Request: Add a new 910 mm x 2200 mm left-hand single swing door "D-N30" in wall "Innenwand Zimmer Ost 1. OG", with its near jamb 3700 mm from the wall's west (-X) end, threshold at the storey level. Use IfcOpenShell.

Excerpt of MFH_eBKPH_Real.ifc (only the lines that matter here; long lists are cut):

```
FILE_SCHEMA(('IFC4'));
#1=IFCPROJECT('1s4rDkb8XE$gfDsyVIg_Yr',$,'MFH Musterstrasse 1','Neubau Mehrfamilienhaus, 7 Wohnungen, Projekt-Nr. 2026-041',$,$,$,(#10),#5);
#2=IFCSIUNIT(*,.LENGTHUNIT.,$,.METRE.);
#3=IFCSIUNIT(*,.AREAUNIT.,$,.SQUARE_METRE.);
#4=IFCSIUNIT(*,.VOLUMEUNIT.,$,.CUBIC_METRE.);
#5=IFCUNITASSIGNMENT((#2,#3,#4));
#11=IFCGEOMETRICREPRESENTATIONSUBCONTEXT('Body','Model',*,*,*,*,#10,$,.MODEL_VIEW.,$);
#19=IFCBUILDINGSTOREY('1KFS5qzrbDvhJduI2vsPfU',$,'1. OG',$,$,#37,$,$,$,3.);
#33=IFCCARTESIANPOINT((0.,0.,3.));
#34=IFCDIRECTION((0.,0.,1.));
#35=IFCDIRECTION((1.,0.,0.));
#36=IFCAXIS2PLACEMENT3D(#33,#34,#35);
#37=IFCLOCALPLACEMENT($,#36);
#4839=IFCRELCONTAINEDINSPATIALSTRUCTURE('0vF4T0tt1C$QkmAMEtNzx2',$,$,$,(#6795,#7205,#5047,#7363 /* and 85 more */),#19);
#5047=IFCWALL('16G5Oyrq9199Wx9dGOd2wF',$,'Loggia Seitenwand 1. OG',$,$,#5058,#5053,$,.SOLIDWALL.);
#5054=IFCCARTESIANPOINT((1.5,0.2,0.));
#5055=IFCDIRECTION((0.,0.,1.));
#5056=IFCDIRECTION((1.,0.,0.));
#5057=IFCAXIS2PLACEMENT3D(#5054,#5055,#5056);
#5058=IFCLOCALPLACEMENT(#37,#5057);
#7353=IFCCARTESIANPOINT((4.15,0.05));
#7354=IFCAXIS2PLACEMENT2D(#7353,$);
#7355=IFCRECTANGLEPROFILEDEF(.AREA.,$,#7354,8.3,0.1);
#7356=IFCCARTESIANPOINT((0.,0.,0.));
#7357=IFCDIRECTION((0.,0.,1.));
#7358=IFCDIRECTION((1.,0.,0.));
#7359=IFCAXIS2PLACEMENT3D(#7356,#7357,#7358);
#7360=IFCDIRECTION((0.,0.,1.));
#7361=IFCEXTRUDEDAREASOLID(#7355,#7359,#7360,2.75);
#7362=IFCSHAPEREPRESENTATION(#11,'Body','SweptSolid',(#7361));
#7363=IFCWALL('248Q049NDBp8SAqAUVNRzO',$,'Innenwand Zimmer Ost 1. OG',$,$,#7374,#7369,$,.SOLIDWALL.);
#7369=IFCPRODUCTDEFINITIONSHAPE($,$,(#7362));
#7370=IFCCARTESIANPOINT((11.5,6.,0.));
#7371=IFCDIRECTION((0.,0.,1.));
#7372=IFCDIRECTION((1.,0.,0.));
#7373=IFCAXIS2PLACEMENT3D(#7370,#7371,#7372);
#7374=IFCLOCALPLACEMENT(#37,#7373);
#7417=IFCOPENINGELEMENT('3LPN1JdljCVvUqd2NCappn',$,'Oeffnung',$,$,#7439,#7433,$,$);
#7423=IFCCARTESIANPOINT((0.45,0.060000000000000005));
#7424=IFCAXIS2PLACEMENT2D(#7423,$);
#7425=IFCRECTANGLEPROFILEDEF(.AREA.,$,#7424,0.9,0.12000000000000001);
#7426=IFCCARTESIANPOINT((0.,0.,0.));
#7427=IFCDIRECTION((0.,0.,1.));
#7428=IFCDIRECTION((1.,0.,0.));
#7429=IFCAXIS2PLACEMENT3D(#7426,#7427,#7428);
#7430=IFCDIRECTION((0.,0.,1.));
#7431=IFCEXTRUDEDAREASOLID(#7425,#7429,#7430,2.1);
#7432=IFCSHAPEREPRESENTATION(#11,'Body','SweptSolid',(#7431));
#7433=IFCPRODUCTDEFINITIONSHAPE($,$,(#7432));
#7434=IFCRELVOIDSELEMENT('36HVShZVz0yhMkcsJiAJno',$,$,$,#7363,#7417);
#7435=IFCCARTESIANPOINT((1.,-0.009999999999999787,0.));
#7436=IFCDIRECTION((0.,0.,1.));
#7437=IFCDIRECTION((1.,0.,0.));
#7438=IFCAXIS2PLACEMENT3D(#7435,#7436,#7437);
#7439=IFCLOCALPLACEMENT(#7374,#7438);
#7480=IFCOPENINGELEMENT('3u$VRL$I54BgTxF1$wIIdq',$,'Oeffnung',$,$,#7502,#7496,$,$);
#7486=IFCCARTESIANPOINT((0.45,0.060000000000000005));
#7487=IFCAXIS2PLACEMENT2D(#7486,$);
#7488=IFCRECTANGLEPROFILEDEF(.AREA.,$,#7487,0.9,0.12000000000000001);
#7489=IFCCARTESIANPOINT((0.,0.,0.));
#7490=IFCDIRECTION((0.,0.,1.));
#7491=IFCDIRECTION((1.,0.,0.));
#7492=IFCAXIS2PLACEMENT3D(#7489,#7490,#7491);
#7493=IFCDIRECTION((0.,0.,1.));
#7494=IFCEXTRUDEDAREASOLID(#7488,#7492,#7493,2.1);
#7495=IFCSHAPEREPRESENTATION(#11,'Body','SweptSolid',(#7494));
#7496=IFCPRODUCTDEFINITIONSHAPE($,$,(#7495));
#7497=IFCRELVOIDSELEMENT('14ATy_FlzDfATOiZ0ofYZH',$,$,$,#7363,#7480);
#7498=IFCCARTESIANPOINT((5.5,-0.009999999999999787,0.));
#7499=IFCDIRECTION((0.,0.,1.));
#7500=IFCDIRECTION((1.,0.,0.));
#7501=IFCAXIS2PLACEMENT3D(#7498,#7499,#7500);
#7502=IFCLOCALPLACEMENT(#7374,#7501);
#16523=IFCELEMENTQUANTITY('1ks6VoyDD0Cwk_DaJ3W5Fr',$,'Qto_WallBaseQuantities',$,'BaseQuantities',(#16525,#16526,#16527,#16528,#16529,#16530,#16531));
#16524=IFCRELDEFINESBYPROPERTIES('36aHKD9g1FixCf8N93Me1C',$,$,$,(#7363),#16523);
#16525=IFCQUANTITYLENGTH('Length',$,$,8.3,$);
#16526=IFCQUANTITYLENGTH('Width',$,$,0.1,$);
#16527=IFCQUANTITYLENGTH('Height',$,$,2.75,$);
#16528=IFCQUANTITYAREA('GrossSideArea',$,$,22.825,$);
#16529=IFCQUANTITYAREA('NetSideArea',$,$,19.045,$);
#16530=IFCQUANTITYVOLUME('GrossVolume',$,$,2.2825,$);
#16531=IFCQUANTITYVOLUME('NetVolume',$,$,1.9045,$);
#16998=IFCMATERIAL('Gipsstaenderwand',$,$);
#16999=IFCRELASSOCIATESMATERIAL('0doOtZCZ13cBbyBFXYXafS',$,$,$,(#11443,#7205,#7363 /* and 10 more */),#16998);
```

```python
import numpy as np
import ifcopenshell
import ifcopenshell.api.feature
import ifcopenshell.api.geometry
import ifcopenshell.api.pset
import ifcopenshell.api.root
import ifcopenshell.api.spatial
import ifcopenshell.geom
import ifcopenshell.util.element
import ifcopenshell.util.placement
import ifcopenshell.util.representation
import ifcopenshell.util.shape
import ifcopenshell.util.unit

model = ifcopenshell.open("MFH_eBKPH_Real.ifc")
unit_scale = ifcopenshell.util.unit.calculate_unit_scale(model)
area_scale = ifcopenshell.util.unit.calculate_unit_scale(model, "AREAUNIT")
volume_scale = ifcopenshell.util.unit.calculate_unit_scale(model, "VOLUMEUNIT")
settings = ifcopenshell.geom.settings()


def volume(element):
    """Net volume in cubic metres, openings subtracted."""
    shape = ifcopenshell.geom.create_shape(settings, element)
    return ifcopenshell.util.shape.get_volume(shape.geometry)


wall = model.by_id(7363)
storey = ifcopenshell.util.element.get_container(wall, ifc_class="IfcBuildingStorey")
context = ifcopenshell.util.representation.get_context(model, "Model", "Body", "MODEL_VIEW")
before = volume(wall)

width, height, from_end, sill = 0.91, 2.2, 3.7, 0.0  # metres

# The wall runs along its own X axis, and the end named is its -X end.
wall_shape = ifcopenshell.geom.create_shape(settings, wall)
x, y, z = ifcopenshell.util.shape.get_vertices(wall_shape.geometry).T
start = x.min() + from_end
face, thickness = float(y.min()), float(y.max() - y.min())
wall_matrix = ifcopenshell.util.placement.get_local_placement(wall.ObjectPlacement)
level = ifcopenshell.util.placement.get_local_placement(storey.ObjectPlacement)[2, 3]


def in_wall(x, y):
    """Placement at x, y metres in the wall's axes, at sill height."""
    matrix = wall_matrix.copy()
    matrix[:, 3] = wall_matrix @ np.array([x / unit_scale, y / unit_scale, 0.0, 1.0])
    matrix[2, 3] = level + sill / unit_scale
    return matrix


# Opening: a box that overshoots both wall faces by 50 mm.
opening = ifcopenshell.api.root.create_entity(model, ifc_class="IfcOpeningElement", predefined_type="OPENING")
box = ifcopenshell.api.geometry.add_wall_representation(
    model, context=context, length=width, height=height, thickness=thickness + 0.1
)
ifcopenshell.api.geometry.assign_representation(model, product=opening, representation=box)
ifcopenshell.api.geometry.edit_object_placement(model, product=opening, matrix=in_wall(start, face - 0.05), is_si=False)
ifcopenshell.api.feature.add_feature(model, feature=opening, element=wall)

door = ifcopenshell.api.root.create_entity(model, ifc_class="IfcDoor", name="D-N30", predefined_type="DOOR")
door.OverallWidth, door.OverallHeight = width / unit_scale, height / unit_scale
door.OperationType = "SINGLE_SWING_LEFT"
body = ifcopenshell.api.geometry.add_door_representation(
    model,
    context=context,
    overall_width=door.OverallWidth,
    overall_height=door.OverallHeight,
    operation_type="SINGLE_SWING_LEFT",
    lining_properties={"LiningDepth": thickness / unit_scale, "ThresholdDepth": thickness / unit_scale},
)
ifcopenshell.api.geometry.assign_representation(model, product=door, representation=body)
ifcopenshell.api.spatial.assign_container(model, products=[door], relating_structure=storey)
ifcopenshell.api.feature.add_filling(model, opening=opening, element=door)

# The lining spans the wall, so the door starts at the wall face.
ifcopenshell.api.geometry.edit_object_placement(model, product=door, matrix=in_wall(start, face), is_si=False)

after = volume(wall)

# Update the wall's stored quantities.
qto = model.by_id(ifcopenshell.util.element.get_pset(wall, "Qto_WallBaseQuantities", should_inherit=False)["id"])
ifcopenshell.api.pset.edit_qto(model, qto=qto, properties={
    "NetSideArea": after / thickness / area_scale,
    "NetVolume": after / volume_scale,
})

print(f"wall volume {before:.3f} -> {after:.3f} m3")

model.write("MFH_eBKPH_Real-out.ifc")
```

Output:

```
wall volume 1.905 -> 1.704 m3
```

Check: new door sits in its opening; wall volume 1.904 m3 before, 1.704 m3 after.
